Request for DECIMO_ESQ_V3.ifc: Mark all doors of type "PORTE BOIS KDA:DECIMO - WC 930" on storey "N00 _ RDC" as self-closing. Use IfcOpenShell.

First a look at what the model holds.

```python
import ifcopenshell
import ifcopenshell.util.element

model = ifcopenshell.open("DECIMO_ESQ_V3.ifc")
print(model.schema)
storey = next(s for s in model.by_type("IfcBuildingStorey") if s.Name == "N00 _ RDC")
doors = [e for e in ifcopenshell.util.element.get_decomposition(storey) if e.is_a("IfcDoor")]
seen = {}
for e in doors:
    element_type = ifcopenshell.util.element.get_type(e)
    key = (element_type.Name if element_type != e and element_type else None, ifcopenshell.util.element.get_pset(e, "Pset_DoorCommon", "SelfClosing"))
    seen[key] = seen.get(key, 0) + 1
for (name, value), count in sorted(seen.items(), key=str):
    print(count, "x", name, "|", value)
```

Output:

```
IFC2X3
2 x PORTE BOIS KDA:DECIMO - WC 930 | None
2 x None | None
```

```python
import ifcopenshell
import ifcopenshell.api.pset
import ifcopenshell.util.element

model = ifcopenshell.open("DECIMO_ESQ_V3.ifc")

storey = next(s for s in model.by_type("IfcBuildingStorey") if s.Name == "N00 _ RDC")
doors = [e for e in ifcopenshell.util.element.get_decomposition(storey) if e.is_a("IfcDoor")]

count = 0
for e in doors:
    element_type = ifcopenshell.util.element.get_type(e)
    if element_type in (None, e) or element_type.Name != "PORTE BOIS KDA:DECIMO - WC 930":
        continue
    # add_pset returns the element's existing set when there is one.
    pset = ifcopenshell.api.pset.add_pset(model, product=e, name="Pset_DoorCommon")
    ifcopenshell.api.pset.edit_pset(model, pset=pset, properties={"SelfClosing": True})
    count += 1

print(count, "doors updated")

model.write("DECIMO_ESQ_V3_v2.ifc")
```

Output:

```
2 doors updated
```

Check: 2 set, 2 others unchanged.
